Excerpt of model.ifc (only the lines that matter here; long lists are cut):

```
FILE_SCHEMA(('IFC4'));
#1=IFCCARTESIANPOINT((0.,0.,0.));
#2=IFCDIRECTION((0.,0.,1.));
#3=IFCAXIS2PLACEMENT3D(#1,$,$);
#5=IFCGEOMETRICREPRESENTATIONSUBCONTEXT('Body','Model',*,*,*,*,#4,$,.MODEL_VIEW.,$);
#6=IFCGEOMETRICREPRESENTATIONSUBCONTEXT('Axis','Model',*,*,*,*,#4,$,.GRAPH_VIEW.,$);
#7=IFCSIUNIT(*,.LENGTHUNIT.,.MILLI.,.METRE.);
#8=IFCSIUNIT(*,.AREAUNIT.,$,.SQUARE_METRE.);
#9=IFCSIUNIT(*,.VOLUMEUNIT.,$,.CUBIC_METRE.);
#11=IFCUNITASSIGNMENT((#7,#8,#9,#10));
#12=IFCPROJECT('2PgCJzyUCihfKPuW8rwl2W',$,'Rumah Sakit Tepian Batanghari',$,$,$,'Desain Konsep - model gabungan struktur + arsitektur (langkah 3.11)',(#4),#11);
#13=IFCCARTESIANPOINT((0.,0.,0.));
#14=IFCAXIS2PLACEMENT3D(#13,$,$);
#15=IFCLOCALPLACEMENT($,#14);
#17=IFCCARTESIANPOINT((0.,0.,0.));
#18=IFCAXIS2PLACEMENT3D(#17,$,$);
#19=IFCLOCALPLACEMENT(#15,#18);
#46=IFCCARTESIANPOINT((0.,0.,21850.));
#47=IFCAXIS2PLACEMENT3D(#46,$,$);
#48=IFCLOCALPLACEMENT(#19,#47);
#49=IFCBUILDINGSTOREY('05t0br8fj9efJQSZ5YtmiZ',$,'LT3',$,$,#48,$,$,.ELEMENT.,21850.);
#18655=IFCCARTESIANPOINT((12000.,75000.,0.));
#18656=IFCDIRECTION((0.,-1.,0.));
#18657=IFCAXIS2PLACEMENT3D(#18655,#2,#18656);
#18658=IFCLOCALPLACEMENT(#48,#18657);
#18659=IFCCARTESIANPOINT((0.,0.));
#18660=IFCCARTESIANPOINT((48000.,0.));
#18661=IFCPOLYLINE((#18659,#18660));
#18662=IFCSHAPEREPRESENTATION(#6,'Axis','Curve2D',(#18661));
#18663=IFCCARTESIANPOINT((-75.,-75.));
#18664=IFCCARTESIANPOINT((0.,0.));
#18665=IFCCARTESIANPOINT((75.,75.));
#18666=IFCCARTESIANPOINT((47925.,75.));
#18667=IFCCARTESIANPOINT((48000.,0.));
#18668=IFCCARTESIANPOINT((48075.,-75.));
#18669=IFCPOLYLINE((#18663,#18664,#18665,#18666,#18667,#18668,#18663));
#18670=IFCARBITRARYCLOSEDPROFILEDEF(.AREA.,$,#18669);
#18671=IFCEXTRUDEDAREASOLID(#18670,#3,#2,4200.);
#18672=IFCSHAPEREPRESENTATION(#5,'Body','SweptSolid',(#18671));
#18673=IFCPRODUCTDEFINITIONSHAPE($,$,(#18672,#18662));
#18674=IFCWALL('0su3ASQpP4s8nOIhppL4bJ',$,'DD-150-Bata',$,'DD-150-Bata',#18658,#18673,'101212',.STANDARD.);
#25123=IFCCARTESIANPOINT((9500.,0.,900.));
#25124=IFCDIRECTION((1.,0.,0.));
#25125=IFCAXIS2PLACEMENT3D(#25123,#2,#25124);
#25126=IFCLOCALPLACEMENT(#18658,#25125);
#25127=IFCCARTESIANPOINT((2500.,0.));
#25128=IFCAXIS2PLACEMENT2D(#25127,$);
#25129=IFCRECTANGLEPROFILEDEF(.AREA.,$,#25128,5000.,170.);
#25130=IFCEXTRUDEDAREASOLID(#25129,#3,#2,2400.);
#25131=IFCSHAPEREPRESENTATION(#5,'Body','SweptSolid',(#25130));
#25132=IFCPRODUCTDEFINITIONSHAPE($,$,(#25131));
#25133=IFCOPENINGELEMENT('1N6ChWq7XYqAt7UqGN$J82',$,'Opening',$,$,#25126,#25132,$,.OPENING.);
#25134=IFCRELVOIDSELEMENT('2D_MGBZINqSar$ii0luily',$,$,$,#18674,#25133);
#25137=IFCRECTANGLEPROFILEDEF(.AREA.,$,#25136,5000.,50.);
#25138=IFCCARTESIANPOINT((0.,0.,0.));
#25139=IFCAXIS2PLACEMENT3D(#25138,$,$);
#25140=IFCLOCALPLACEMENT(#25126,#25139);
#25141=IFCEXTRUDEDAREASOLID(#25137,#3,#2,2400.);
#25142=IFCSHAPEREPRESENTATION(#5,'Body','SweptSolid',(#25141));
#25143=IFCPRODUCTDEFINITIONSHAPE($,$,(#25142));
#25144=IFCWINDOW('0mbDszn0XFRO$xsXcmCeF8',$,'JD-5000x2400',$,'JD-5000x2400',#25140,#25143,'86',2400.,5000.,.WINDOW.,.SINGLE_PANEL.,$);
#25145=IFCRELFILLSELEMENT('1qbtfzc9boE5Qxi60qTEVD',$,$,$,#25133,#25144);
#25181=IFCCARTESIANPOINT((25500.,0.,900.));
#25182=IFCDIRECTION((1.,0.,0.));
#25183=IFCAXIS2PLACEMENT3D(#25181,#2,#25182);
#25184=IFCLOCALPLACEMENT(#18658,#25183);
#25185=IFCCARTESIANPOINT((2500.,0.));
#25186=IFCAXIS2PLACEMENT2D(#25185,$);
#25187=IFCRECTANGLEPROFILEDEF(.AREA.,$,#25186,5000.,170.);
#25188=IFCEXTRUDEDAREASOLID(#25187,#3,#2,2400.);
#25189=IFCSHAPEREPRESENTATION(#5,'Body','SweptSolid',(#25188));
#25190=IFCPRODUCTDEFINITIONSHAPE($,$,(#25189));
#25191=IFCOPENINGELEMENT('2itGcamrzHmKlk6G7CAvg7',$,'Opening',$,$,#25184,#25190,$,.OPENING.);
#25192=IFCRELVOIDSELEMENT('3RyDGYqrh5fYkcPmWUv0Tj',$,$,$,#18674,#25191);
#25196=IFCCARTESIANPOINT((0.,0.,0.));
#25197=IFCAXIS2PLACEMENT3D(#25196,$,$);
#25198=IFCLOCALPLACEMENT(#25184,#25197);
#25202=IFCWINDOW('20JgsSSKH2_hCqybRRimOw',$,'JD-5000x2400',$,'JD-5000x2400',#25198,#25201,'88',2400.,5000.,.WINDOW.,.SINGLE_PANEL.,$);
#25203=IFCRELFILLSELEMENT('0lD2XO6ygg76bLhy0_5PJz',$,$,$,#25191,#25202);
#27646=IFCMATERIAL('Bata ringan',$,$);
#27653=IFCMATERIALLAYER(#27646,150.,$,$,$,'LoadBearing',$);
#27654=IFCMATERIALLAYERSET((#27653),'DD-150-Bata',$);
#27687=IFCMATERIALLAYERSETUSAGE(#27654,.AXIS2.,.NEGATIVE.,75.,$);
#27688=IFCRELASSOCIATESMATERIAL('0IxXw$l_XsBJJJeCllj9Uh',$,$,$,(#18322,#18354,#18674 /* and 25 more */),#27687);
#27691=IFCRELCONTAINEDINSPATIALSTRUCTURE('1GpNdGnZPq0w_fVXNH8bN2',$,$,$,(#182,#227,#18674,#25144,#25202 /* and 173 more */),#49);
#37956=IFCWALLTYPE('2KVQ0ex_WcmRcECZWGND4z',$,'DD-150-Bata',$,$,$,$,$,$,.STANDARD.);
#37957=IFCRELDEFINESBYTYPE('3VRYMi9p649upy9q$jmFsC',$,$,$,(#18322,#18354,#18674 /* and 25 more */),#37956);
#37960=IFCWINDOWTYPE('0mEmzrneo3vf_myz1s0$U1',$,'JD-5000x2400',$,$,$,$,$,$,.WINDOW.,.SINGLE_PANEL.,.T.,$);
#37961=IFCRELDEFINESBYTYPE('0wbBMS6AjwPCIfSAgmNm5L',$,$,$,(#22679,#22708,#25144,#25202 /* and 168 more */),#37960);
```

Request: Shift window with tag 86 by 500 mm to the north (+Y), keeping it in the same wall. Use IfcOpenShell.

```python
import ifcopenshell
import ifcopenshell.api.geometry
import ifcopenshell.util.placement
import ifcopenshell.util.unit

model = ifcopenshell.open("model.ifc")
unit_scale = ifcopenshell.util.unit.calculate_unit_scale(model)

window = model.by_guid("0mbDszn0XFRO$xsXcmCeF8")
opening = window.FillsVoids[0].RelatingOpeningElement
wall = opening.VoidsElements[0].RelatingBuildingElement

wall_matrix = ifcopenshell.util.placement.get_local_placement(wall.ObjectPlacement)
shift = wall_matrix[:3, 0] * -0.5 / unit_scale
before = ifcopenshell.util.placement.get_local_placement(window.ObjectPlacement)[:3, 3].copy()

# The window is placed relative to its opening, so it follows when the opening moves.
matrix = ifcopenshell.util.placement.get_local_placement(opening.ObjectPlacement)
matrix[:3, 3] += shift
ifcopenshell.api.geometry.edit_object_placement(
    model, product=opening, matrix=matrix, is_si=False, should_transform_children=True
)

after = ifcopenshell.util.placement.get_local_placement(window.ObjectPlacement)[:3, 3]
print("window moved by", (after - before).round(3) + 0.0)

model.write("model-out.ifc")
```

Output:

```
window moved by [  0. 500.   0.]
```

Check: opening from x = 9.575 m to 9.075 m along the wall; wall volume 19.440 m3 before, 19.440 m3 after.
